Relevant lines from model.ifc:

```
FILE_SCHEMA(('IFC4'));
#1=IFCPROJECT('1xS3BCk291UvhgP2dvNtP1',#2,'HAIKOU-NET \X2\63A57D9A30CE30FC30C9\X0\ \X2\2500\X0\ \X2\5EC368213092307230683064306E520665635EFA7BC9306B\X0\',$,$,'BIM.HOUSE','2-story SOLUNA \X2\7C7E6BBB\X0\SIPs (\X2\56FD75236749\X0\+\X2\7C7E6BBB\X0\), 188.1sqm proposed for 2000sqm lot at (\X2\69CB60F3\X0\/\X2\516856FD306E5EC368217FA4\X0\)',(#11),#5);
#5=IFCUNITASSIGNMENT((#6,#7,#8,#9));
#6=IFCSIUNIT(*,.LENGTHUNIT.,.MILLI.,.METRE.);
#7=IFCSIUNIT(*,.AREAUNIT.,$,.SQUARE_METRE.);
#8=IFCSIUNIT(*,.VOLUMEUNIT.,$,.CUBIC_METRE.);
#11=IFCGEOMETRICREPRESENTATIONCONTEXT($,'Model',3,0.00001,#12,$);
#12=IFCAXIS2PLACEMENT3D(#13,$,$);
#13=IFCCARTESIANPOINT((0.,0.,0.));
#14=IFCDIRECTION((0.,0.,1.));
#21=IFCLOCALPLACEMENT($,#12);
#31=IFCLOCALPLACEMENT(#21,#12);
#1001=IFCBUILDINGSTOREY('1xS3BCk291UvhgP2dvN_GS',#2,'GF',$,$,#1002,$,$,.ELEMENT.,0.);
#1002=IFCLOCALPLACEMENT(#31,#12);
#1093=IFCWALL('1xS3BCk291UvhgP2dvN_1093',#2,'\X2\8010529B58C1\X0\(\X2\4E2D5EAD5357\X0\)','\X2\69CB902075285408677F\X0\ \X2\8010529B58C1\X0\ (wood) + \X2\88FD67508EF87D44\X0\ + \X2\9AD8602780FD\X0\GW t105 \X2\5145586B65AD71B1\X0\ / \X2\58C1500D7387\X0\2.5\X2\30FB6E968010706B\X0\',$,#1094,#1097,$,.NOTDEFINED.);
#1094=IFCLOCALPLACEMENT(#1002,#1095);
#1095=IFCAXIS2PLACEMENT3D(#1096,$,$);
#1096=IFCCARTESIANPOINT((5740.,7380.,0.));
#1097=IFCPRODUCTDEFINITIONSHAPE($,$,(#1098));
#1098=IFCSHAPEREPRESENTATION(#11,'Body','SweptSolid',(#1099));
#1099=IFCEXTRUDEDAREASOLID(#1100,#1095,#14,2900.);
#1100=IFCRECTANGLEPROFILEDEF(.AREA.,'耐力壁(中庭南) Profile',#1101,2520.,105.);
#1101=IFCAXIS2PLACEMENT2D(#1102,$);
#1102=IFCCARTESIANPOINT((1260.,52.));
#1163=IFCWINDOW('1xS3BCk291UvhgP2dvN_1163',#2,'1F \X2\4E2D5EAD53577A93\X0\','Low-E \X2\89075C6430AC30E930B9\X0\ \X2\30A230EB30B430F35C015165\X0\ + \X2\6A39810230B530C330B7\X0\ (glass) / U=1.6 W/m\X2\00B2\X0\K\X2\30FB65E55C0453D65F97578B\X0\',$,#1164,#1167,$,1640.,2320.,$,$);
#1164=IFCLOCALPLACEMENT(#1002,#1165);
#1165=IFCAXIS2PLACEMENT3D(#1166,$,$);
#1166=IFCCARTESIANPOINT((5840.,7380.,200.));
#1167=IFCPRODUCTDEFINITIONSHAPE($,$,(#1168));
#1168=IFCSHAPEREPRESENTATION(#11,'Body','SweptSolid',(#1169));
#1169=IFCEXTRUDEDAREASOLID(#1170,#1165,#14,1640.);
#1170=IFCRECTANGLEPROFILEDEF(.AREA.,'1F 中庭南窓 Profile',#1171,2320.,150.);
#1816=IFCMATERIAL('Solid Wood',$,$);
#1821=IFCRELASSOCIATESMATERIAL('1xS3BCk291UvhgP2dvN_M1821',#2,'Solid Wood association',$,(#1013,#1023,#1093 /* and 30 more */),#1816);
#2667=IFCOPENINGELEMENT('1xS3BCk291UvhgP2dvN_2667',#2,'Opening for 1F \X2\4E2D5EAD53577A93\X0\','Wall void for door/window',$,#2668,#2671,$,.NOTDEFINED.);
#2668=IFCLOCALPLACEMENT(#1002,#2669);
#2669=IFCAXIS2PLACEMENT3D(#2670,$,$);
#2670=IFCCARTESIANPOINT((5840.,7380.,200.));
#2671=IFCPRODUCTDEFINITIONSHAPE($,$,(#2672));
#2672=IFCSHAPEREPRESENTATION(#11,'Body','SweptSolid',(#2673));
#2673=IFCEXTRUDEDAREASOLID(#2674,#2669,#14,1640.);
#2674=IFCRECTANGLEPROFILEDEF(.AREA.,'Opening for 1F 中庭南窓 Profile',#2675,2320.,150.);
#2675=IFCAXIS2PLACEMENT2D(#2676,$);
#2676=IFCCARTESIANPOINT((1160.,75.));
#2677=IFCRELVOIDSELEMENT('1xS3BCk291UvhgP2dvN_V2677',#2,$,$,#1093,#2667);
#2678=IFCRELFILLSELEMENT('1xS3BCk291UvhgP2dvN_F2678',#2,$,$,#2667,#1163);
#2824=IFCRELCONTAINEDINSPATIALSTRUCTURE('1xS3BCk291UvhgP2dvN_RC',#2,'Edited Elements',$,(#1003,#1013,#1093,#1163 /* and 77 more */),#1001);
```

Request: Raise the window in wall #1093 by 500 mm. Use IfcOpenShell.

```python
import numpy as np
import ifcopenshell
import ifcopenshell.api.geometry
import ifcopenshell.util.placement
import ifcopenshell.util.unit

model = ifcopenshell.open("model.ifc")
unit_scale = ifcopenshell.util.unit.calculate_unit_scale(model)

window = model.by_guid("1xS3BCk291UvhgP2dvN_1163")
opening = window.FillsVoids[0].RelatingOpeningElement
dz = 0.5 / unit_scale

shift = np.array([0.0, 0.0, dz])
# The window is not placed relative to its opening, so move both.
for product in (opening, window):
    matrix = ifcopenshell.util.placement.get_local_placement(product.ObjectPlacement)
    matrix[:3, 3] += shift
    ifcopenshell.api.geometry.edit_object_placement(model, product=product, matrix=matrix, is_si=False)

print(f"moved by {dz * unit_scale:+.3f} m")

model.write("model_updated.ifc")
```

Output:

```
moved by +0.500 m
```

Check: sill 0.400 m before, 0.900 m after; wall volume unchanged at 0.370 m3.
